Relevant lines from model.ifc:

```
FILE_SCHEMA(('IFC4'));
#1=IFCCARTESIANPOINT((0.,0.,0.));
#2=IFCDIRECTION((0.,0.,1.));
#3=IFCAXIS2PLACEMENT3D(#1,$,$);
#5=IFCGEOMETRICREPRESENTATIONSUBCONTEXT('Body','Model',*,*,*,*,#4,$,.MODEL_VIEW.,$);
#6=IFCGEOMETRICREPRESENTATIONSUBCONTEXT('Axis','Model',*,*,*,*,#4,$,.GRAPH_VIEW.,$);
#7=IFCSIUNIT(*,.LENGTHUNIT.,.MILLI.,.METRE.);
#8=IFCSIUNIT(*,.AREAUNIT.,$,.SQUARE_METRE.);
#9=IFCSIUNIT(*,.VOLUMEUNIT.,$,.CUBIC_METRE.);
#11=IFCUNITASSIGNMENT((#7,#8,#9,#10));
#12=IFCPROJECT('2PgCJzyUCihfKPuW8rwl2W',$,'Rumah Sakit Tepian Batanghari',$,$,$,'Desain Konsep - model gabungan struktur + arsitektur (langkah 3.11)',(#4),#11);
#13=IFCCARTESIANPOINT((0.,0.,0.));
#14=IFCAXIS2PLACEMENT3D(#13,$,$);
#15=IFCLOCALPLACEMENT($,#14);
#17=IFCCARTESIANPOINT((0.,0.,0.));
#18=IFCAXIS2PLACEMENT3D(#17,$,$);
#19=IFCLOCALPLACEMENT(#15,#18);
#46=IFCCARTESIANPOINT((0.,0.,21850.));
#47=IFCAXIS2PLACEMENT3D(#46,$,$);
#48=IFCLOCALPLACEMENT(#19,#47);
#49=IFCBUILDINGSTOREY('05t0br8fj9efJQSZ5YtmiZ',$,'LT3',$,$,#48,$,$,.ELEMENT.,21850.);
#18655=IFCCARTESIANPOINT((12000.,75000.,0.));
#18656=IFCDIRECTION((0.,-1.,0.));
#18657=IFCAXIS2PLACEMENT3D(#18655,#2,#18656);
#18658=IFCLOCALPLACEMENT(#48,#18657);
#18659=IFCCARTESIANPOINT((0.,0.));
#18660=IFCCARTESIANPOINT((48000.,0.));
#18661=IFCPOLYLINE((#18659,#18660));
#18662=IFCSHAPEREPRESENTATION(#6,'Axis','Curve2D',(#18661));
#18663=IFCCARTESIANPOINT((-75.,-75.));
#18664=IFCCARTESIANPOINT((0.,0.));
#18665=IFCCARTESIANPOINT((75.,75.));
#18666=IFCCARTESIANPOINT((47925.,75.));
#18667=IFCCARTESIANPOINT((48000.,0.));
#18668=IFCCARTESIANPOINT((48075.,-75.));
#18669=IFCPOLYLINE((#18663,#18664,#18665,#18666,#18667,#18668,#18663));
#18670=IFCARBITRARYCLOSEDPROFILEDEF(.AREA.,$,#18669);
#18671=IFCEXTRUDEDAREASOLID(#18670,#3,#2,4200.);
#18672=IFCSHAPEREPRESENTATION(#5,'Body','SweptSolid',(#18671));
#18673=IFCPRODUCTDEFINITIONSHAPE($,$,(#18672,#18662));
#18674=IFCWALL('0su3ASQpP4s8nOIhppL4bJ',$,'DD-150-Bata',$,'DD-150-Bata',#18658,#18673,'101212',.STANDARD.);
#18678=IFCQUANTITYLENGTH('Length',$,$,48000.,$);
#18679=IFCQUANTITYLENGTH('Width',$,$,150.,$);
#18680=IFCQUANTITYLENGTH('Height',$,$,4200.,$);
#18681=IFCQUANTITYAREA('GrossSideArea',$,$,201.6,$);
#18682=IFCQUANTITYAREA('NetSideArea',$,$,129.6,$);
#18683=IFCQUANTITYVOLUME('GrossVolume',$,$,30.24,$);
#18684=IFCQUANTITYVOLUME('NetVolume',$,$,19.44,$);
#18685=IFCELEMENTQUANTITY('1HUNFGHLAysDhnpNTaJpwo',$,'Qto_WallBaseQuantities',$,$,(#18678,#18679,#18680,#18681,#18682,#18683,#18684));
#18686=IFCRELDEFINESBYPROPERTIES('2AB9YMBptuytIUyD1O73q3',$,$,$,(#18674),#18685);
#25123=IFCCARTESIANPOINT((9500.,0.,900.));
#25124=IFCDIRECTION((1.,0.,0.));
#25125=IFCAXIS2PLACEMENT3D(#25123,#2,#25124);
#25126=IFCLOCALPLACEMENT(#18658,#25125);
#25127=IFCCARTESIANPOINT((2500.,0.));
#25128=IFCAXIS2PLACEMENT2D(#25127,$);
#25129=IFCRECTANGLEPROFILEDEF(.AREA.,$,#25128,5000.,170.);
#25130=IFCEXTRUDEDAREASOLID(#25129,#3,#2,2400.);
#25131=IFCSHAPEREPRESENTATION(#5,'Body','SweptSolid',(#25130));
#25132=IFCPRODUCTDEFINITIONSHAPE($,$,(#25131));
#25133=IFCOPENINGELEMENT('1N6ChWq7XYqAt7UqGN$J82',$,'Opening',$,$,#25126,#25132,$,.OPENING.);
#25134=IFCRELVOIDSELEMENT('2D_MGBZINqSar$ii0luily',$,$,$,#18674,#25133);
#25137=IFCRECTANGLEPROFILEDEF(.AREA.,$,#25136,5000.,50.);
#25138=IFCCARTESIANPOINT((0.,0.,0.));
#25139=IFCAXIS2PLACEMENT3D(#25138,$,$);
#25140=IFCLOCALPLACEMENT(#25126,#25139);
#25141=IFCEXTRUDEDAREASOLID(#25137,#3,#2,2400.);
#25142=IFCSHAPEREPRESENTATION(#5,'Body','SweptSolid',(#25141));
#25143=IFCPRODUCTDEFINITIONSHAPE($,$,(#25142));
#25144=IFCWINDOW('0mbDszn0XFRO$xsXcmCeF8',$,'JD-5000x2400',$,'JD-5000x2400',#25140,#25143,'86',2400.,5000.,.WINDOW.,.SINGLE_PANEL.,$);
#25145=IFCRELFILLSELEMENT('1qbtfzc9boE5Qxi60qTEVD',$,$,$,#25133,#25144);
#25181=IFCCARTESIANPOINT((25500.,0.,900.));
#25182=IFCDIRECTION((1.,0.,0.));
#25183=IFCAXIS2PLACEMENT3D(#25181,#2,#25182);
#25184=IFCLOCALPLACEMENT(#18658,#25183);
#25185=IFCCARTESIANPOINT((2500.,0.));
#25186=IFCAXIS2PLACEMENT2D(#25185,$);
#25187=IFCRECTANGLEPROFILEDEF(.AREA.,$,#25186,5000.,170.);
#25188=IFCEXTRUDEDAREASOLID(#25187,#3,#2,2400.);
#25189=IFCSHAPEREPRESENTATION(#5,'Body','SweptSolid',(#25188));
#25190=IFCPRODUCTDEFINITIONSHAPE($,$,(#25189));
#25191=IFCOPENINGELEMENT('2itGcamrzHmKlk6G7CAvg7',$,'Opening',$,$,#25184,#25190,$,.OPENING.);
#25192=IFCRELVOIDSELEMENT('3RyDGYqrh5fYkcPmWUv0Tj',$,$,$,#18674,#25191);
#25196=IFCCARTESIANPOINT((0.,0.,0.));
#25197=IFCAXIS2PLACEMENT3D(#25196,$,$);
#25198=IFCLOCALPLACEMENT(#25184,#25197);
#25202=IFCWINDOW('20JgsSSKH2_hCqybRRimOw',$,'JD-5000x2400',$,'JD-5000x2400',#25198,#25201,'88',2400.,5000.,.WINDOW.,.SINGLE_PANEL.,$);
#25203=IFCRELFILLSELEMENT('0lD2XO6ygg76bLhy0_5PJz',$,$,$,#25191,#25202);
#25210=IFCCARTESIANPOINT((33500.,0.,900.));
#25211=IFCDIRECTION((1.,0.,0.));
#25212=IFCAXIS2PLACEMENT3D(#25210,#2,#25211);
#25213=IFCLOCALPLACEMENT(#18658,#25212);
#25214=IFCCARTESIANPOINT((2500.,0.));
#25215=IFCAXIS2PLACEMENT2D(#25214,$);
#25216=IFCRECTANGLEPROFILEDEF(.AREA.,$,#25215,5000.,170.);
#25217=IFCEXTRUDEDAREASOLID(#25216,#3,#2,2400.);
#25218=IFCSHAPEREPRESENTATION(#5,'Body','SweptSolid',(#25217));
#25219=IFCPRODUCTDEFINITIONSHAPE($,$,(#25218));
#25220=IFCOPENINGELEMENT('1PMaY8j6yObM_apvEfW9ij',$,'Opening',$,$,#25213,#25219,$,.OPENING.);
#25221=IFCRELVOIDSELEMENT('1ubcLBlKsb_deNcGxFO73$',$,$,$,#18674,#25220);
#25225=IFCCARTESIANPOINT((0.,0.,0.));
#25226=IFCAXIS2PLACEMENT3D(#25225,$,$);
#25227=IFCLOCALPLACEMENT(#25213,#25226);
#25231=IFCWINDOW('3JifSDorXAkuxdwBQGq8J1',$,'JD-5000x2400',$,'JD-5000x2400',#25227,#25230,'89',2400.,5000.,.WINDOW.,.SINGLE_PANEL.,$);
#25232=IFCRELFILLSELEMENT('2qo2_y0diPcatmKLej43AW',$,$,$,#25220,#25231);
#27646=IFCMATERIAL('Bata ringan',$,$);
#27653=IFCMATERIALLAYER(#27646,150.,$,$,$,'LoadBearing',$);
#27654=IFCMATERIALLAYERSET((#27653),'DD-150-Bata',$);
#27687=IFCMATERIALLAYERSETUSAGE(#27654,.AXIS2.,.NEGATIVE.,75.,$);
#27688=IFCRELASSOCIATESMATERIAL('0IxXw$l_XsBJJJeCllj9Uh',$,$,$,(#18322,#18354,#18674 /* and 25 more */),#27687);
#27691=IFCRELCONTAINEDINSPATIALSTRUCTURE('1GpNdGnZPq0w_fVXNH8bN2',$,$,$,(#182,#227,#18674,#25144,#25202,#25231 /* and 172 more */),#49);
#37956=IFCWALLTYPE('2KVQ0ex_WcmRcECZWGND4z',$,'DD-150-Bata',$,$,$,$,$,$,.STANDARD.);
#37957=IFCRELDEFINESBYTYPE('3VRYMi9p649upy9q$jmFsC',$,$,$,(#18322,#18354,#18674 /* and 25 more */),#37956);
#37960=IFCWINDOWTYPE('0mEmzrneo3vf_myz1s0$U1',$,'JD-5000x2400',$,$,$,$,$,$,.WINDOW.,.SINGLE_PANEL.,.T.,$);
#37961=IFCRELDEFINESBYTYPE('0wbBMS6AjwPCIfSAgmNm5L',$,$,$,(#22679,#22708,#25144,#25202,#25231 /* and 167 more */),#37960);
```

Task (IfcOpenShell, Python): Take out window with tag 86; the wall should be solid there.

```python
import ifcopenshell
import ifcopenshell.api.feature
import ifcopenshell.api.pset
import ifcopenshell.api.root
import ifcopenshell.geom
import ifcopenshell.util.element
import ifcopenshell.util.shape
import ifcopenshell.util.unit

model = ifcopenshell.open("model.ifc")
area_scale = ifcopenshell.util.unit.calculate_unit_scale(model, "AREAUNIT")
volume_scale = ifcopenshell.util.unit.calculate_unit_scale(model, "VOLUMEUNIT")
settings = ifcopenshell.geom.settings()


def volume(element):
    """Net volume in cubic metres, openings subtracted."""
    shape = ifcopenshell.geom.create_shape(settings, element)
    return ifcopenshell.util.shape.get_volume(shape.geometry)


window = model.by_guid("0mbDszn0XFRO$xsXcmCeF8")
opening = window.FillsVoids[0].RelatingOpeningElement
wall = opening.VoidsElements[0].RelatingBuildingElement
before = volume(wall)

ifcopenshell.api.root.remove_product(model, product=window)
ifcopenshell.api.feature.remove_feature(model, feature=opening)

after = volume(wall)
thickness = 0.15  # wall thickness in metres

# Update the wall's stored quantities.
qto = model.by_id(ifcopenshell.util.element.get_pset(wall, "Qto_WallBaseQuantities", should_inherit=False)["id"])
ifcopenshell.api.pset.edit_qto(model, qto=qto, properties={
    "NetSideArea": after / thickness / area_scale,
    "NetVolume": after / volume_scale,
})

print(f"wall volume {before:.3f} -> {after:.3f} m3")

model.write("model_v2.ifc")
```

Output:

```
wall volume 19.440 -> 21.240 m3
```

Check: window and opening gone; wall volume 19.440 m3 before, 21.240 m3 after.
